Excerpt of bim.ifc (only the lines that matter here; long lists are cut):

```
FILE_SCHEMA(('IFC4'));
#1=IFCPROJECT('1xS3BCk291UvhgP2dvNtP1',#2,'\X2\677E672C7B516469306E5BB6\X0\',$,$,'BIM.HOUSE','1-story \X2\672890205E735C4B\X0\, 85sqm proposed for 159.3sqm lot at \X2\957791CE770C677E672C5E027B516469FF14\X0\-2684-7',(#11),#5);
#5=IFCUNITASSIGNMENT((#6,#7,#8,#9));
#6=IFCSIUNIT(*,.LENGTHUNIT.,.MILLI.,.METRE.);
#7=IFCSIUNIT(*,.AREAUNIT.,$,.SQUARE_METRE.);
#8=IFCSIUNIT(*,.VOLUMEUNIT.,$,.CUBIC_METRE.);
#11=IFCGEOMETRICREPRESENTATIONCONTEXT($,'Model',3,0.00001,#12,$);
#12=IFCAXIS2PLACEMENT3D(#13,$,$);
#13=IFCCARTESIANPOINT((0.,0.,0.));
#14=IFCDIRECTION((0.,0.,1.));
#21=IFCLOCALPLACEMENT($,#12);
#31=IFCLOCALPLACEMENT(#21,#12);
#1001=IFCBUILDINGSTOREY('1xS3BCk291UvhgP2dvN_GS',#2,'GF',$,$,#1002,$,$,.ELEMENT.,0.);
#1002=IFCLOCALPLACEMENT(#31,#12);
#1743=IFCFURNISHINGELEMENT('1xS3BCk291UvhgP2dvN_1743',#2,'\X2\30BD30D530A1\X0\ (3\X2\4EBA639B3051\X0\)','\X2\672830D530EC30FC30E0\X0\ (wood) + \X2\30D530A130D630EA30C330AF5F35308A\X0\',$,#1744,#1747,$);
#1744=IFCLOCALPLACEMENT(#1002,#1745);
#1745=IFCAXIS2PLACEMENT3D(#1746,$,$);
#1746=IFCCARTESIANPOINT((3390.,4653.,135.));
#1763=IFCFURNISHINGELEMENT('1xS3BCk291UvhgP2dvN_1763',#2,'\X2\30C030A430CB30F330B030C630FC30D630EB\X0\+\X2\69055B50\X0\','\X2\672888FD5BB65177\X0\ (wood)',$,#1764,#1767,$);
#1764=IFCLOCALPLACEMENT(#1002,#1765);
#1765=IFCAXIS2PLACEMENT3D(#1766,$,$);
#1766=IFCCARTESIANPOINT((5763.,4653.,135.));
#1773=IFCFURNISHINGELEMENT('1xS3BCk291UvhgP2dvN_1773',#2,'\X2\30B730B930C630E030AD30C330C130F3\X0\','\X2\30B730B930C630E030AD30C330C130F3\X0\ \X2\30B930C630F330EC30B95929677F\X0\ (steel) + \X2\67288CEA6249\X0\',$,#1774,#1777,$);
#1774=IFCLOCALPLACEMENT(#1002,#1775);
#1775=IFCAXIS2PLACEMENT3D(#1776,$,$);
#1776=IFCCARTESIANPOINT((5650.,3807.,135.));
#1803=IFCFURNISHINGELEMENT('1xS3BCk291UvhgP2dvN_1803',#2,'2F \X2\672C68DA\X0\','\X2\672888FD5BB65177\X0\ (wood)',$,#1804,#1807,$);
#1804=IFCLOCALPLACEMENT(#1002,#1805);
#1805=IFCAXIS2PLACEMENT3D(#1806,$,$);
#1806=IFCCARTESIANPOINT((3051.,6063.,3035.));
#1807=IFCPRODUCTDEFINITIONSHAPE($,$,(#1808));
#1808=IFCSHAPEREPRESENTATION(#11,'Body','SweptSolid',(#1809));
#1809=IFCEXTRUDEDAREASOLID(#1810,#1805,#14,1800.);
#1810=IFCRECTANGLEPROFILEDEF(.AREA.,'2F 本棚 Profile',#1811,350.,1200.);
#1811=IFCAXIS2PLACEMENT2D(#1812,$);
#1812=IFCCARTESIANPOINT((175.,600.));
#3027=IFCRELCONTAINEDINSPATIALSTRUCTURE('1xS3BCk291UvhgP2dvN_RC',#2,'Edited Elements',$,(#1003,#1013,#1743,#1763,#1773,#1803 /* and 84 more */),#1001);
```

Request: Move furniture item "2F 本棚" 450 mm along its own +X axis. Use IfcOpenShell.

```python
import ifcopenshell
import ifcopenshell.api.geometry
import ifcopenshell.util.placement
import ifcopenshell.util.unit

model = ifcopenshell.open("bim.ifc")
unit_scale = ifcopenshell.util.unit.calculate_unit_scale(model)

item = model.by_guid("1xS3BCk291UvhgP2dvN_1803")
matrix = ifcopenshell.util.placement.get_local_placement(item.ObjectPlacement)
matrix[:3, 3] += matrix[:3, 0] * 0.45 / unit_scale
ifcopenshell.api.geometry.edit_object_placement(model, product=item, matrix=matrix, is_si=False)

print(ifcopenshell.util.placement.get_local_placement(item.ObjectPlacement).round(3) + 0.0)

model.write("bim-out.ifc")
```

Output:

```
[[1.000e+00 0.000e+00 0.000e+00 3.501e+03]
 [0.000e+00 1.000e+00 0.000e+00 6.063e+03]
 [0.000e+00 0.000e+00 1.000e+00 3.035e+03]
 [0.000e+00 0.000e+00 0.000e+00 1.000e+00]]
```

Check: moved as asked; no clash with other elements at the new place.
